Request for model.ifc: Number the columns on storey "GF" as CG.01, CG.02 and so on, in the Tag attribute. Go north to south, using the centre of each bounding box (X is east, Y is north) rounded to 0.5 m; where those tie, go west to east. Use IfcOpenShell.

First a look at what the model holds.

```python
import ifcopenshell
import ifcopenshell.util.element
import ifcopenshell.util.placement

model = ifcopenshell.open("model.ifc")
print(model.schema)
storey = next(s for s in model.by_type("IfcBuildingStorey") if s.Name == "GF")
columns = [e for e in ifcopenshell.util.element.get_decomposition(storey) if e.is_a("IfcColumn")]
for e in sorted(columns, key=lambda e: e.id()):
    origin = ifcopenshell.util.placement.get_local_placement(e.ObjectPlacement)[:3, 3]
    print(e.id(), e.Tag, e.Name, origin.round(2) + 0.0, sep=" | ")
```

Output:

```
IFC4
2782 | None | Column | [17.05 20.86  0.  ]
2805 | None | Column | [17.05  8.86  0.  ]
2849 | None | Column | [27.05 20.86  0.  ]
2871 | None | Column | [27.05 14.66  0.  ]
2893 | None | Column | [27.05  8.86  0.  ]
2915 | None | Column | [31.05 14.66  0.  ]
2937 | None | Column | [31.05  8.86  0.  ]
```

```python
import ifcopenshell
import ifcopenshell.geom
import ifcopenshell.util.element
import ifcopenshell.util.shape

model = ifcopenshell.open("model.ifc")
settings = ifcopenshell.geom.settings()
settings.set("use-world-coords", True)


def centre(element):
    shape = ifcopenshell.geom.create_shape(settings, element)
    return ifcopenshell.util.shape.get_bbox_centroid(shape.geometry)


storey = next(s for s in model.by_type("IfcBuildingStorey") if s.Name == "GF")
columns = [e for e in ifcopenshell.util.element.get_decomposition(storey) if e.is_a("IfcColumn")]

# Insertion points can sit at a corner or the storey origin, so sort by the geometry (in metres).
centres = {e: centre(e) for e in columns}
columns.sort(key=lambda e: (-round(centres[e][1] / 0.5), centres[e][0]))

for i, e in enumerate(columns, start=1):
    number = f"CG.{i:02d}"
    e.Tag = number
    print(e.id(), number)

model.write("model_edited.ifc")
```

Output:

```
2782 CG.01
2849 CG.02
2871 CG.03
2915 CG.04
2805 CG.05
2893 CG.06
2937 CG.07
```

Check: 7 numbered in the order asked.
